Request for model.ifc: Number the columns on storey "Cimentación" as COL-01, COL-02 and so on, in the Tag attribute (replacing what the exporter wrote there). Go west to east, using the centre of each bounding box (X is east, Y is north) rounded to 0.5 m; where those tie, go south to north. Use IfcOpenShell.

First a look at what the model holds.

```python
import ifcopenshell
import ifcopenshell.util.element
import ifcopenshell.util.placement

model = ifcopenshell.open("model.ifc")
print(model.schema)
storey = next(s for s in model.by_type("IfcBuildingStorey") if s.Name == "Cimentación")
columns = [e for e in ifcopenshell.util.element.get_decomposition(storey) if e.is_a("IfcColumn")]
for e in sorted(columns, key=lambda e: e.id()):
    origin = ifcopenshell.util.placement.get_local_placement(e.ObjectPlacement)[:3, 3]
    print(e.id(), e.Tag, e.Name, origin.round(2) + 0.0, sep=" | ")
```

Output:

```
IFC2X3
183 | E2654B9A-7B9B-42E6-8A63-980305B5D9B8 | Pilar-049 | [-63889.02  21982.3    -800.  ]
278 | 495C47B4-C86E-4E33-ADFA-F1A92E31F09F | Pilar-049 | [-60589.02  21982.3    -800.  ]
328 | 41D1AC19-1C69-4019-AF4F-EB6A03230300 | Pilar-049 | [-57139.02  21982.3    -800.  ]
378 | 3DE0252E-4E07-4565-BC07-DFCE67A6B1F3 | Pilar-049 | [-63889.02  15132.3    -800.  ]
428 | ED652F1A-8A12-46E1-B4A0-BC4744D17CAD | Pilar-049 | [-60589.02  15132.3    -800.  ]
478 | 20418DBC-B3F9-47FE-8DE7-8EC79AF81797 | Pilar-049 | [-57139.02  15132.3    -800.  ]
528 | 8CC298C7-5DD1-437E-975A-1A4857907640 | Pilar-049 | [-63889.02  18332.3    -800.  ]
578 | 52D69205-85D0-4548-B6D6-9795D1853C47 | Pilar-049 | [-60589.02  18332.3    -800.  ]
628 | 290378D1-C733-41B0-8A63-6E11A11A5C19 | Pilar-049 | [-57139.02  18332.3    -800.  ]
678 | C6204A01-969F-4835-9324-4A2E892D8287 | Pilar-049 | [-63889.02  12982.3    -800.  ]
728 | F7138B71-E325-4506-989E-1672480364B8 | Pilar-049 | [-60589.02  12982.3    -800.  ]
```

```python
import ifcopenshell
import ifcopenshell.geom
import ifcopenshell.util.element
import ifcopenshell.util.shape

model = ifcopenshell.open("model.ifc")
settings = ifcopenshell.geom.settings()
settings.set("use-world-coords", True)


def centre(element):
    shape = ifcopenshell.geom.create_shape(settings, element)
    return ifcopenshell.util.shape.get_bbox_centroid(shape.geometry)


storey = next(s for s in model.by_type("IfcBuildingStorey") if s.Name == "Cimentación")
columns = [e for e in ifcopenshell.util.element.get_decomposition(storey) if e.is_a("IfcColumn")]

# Insertion points can sit at a corner or the storey origin, so sort by the geometry (in metres).
centres = {e: centre(e) for e in columns}
columns.sort(key=lambda e: (round(centres[e][0] / 0.5), centres[e][1]))

for i, e in enumerate(columns, start=1):
    number = f"COL-{i:02d}"
    e.Tag = number
    print(e.id(), number)

model.write("model_v2.ifc")
```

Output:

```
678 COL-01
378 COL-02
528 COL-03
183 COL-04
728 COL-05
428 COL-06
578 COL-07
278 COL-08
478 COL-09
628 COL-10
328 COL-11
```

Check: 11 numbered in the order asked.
